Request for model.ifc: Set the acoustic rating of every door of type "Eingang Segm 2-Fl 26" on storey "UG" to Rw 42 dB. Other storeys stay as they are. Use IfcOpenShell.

First a look at what the model holds.

```python
import ifcopenshell
import ifcopenshell.util.element

model = ifcopenshell.open("model.ifc")
print(model.schema)
storey = next(s for s in model.by_type("IfcBuildingStorey") if s.Name == "UG")
doors = [e for e in ifcopenshell.util.element.get_decomposition(storey) if e.is_a("IfcDoor")]
seen = {}
for e in doors:
    element_type = ifcopenshell.util.element.get_type(e)
    key = (element_type.Name if element_type != e and element_type else None, ifcopenshell.util.element.get_pset(e, "Pset_DoorCommon", "AcousticRating"))
    seen[key] = seen.get(key, 0) + 1
for (name, value), count in sorted(seen.items(), key=str):
    print(count, "x", name, "|", value)
```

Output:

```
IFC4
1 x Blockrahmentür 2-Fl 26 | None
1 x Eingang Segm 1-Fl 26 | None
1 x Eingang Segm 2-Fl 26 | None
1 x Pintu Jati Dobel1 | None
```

```python
import ifcopenshell
import ifcopenshell.api.pset
import ifcopenshell.util.element

model = ifcopenshell.open("model.ifc")

storey = next(s for s in model.by_type("IfcBuildingStorey") if s.Name == "UG")
doors = [e for e in ifcopenshell.util.element.get_decomposition(storey) if e.is_a("IfcDoor")]

count = 0
for e in doors:
    element_type = ifcopenshell.util.element.get_type(e)
    if element_type in (None, e) or element_type.Name != "Eingang Segm 2-Fl 26":
        continue
    # add_pset returns the element's existing set when there is one.
    pset = ifcopenshell.api.pset.add_pset(model, product=e, name="Pset_DoorCommon")
    ifcopenshell.api.pset.edit_pset(model, pset=pset, properties={"AcousticRating": "Rw 42 dB"})
    count += 1

print(count, "doors updated")

model.write("model_v2.ifc")
```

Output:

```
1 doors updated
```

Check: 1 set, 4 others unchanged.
